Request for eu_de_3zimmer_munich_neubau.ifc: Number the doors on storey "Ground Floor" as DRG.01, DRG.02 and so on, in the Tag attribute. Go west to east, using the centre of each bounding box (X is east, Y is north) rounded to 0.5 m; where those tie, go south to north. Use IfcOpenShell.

First a look at what the model holds.

```python
import ifcopenshell
import ifcopenshell.util.element
import ifcopenshell.util.placement

model = ifcopenshell.open("eu_de_3zimmer_munich_neubau.ifc")
print(model.schema)
storey = next(s for s in model.by_type("IfcBuildingStorey") if s.Name == "Ground Floor")
doors = [e for e in ifcopenshell.util.element.get_decomposition(storey) if e.is_a("IfcDoor")]
for e in sorted(doors, key=lambda e: e.id()):
    origin = ifcopenshell.util.placement.get_local_placement(e.ObjectPlacement)[:3, 3]
    print(e.id(), e.Tag, e.Name, origin.round(2) + 0.0, sep=" | ")
```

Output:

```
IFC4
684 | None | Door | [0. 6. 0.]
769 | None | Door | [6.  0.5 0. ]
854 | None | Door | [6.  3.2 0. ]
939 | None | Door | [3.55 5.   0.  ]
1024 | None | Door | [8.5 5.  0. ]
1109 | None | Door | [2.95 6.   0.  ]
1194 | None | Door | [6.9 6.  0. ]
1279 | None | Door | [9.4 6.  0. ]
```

```python
import ifcopenshell
import ifcopenshell.geom
import ifcopenshell.util.element
import ifcopenshell.util.shape

model = ifcopenshell.open("eu_de_3zimmer_munich_neubau.ifc")
settings = ifcopenshell.geom.settings()
settings.set("use-world-coords", True)


def centre(element):
    shape = ifcopenshell.geom.create_shape(settings, element)
    return ifcopenshell.util.shape.get_bbox_centroid(shape.geometry)


storey = next(s for s in model.by_type("IfcBuildingStorey") if s.Name == "Ground Floor")
doors = [e for e in ifcopenshell.util.element.get_decomposition(storey) if e.is_a("IfcDoor")]

# Insertion points can sit at a corner or the storey origin, so sort by the geometry (in metres).
centres = {e: centre(e) for e in doors}
doors.sort(key=lambda e: (round(centres[e][0] / 0.5), centres[e][1]))

for i, e in enumerate(doors, start=1):
    number = f"DRG.{i:02d}"
    e.Tag = number
    print(e.id(), number)

model.write("eu_de_3zimmer_munich_neubau_edited.ifc")
```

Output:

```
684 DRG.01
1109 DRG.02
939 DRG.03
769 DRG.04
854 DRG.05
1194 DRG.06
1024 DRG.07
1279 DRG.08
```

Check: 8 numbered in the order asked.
